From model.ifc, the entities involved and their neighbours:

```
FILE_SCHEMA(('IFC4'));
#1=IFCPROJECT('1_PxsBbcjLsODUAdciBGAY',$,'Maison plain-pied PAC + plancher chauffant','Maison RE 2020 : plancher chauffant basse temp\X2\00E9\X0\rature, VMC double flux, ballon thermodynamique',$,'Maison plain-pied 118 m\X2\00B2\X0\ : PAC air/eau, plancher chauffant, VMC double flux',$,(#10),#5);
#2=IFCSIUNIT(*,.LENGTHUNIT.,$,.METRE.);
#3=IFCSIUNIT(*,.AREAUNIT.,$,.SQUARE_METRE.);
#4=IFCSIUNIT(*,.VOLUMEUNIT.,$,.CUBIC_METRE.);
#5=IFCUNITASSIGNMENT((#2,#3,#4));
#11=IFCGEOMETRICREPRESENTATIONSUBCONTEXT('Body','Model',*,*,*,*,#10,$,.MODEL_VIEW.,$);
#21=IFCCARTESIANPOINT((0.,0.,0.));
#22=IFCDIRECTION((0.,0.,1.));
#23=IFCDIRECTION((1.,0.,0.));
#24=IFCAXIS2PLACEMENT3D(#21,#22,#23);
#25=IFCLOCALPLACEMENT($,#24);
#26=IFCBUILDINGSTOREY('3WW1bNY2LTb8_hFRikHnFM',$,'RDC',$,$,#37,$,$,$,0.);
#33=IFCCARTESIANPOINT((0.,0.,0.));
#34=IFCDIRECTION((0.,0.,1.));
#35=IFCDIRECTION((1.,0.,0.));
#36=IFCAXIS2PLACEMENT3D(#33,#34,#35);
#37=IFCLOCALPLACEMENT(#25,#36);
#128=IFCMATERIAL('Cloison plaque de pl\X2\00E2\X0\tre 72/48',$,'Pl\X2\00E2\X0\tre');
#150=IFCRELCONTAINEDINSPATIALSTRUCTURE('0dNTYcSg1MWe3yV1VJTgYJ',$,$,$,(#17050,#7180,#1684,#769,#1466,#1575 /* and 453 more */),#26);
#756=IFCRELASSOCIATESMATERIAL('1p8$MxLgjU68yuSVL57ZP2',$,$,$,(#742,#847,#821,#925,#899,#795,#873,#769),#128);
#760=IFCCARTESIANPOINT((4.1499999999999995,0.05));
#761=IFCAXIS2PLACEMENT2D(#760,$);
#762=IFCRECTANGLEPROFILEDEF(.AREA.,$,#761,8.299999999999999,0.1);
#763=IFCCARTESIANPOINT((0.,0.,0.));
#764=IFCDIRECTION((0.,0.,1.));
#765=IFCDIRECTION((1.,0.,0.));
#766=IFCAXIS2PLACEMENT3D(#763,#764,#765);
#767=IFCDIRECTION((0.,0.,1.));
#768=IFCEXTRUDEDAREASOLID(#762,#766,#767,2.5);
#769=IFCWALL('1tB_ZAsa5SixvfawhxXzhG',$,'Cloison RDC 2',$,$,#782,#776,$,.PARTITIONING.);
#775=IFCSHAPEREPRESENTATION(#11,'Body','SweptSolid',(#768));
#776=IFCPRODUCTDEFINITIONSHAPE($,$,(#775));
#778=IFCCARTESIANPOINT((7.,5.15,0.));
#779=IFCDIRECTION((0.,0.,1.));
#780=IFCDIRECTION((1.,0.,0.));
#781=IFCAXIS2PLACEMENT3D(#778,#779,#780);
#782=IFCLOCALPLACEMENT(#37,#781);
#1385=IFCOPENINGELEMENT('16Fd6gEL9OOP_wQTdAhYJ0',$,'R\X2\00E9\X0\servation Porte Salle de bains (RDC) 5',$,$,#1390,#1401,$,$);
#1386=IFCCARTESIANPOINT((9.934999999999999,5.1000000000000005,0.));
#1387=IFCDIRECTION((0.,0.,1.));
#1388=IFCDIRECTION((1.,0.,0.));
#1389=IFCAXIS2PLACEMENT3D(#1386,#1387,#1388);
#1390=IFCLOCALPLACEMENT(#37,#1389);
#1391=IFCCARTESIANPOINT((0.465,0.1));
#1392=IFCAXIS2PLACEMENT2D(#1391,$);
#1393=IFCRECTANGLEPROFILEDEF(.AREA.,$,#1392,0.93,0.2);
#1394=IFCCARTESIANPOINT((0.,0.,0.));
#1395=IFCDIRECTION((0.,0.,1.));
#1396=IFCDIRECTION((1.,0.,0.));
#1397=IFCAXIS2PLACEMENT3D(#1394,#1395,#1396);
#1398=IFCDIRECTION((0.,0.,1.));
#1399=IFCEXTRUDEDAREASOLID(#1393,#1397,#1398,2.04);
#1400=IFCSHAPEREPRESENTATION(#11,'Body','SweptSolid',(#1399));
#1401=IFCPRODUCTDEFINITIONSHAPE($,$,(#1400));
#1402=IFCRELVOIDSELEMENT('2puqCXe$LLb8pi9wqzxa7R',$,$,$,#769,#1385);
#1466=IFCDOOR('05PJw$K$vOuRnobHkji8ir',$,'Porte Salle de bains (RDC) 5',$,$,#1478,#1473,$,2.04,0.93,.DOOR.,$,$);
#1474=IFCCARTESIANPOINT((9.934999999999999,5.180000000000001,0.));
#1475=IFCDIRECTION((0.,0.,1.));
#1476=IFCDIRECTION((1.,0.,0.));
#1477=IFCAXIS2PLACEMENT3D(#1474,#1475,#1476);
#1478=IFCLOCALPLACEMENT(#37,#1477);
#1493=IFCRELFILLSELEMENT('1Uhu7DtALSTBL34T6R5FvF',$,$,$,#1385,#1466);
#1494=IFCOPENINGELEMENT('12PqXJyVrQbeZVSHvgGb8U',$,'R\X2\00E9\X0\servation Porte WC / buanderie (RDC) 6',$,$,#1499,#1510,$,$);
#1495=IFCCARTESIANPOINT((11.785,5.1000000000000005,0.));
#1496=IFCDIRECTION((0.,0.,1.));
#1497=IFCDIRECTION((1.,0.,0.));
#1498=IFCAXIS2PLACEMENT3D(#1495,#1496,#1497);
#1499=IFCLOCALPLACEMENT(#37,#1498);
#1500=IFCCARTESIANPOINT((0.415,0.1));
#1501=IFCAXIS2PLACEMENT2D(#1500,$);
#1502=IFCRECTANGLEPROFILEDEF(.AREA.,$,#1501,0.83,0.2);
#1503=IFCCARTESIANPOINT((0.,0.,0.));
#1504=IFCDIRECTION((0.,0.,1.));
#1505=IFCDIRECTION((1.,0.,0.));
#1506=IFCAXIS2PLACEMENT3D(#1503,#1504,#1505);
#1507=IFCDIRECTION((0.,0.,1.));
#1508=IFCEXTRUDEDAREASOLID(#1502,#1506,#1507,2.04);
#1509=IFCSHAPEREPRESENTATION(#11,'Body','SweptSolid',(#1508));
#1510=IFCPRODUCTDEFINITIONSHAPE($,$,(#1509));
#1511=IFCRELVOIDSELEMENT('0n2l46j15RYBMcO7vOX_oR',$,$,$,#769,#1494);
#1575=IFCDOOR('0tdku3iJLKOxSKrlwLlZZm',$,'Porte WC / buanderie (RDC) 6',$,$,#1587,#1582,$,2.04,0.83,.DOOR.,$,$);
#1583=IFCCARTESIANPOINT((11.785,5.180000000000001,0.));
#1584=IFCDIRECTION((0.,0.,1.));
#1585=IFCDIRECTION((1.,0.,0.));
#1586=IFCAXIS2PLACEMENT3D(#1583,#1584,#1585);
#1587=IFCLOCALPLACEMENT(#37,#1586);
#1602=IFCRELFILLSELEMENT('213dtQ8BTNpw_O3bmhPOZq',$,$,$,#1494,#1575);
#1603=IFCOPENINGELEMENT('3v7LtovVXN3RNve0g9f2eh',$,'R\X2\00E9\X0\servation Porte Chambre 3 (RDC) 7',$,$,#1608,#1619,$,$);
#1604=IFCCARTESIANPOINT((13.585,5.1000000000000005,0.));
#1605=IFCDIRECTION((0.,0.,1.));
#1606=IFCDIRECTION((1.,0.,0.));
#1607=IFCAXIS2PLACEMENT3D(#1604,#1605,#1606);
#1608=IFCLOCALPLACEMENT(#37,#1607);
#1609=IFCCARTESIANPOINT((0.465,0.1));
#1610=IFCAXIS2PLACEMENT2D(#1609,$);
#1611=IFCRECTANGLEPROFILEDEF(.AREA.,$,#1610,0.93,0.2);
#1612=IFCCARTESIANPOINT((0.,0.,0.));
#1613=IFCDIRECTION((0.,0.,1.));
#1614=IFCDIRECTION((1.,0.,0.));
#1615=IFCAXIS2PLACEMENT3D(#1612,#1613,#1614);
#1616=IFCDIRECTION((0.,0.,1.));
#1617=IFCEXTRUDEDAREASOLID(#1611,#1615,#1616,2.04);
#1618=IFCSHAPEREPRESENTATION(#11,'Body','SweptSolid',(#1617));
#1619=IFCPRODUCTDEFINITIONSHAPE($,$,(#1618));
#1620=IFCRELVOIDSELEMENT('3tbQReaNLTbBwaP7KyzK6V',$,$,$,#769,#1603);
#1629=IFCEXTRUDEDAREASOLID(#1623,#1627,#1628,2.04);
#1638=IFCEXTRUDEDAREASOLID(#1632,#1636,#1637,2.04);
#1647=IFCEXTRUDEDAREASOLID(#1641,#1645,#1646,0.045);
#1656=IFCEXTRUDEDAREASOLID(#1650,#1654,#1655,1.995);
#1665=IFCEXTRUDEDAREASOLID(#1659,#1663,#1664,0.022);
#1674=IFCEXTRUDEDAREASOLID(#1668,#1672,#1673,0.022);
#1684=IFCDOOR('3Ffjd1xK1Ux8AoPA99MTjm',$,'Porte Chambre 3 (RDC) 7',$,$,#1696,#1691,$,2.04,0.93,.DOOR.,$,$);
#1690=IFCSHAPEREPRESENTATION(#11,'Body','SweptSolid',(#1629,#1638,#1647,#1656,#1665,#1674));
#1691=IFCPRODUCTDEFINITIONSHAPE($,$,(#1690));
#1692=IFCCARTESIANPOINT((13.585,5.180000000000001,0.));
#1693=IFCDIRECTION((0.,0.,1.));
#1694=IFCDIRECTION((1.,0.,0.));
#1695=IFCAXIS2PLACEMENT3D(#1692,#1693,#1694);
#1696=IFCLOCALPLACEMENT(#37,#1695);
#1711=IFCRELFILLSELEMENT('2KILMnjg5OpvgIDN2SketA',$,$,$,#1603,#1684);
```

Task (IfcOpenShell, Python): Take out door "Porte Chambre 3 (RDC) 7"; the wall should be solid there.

```python
import ifcopenshell
import ifcopenshell.api.feature
import ifcopenshell.api.root
import ifcopenshell.geom
import ifcopenshell.util.shape

model = ifcopenshell.open("model.ifc")
settings = ifcopenshell.geom.settings()


def volume(element):
    """Net volume in cubic metres, openings subtracted."""
    shape = ifcopenshell.geom.create_shape(settings, element)
    return ifcopenshell.util.shape.get_volume(shape.geometry)


door = model.by_guid("3Ffjd1xK1Ux8AoPA99MTjm")
opening = door.FillsVoids[0].RelatingOpeningElement
wall = opening.VoidsElements[0].RelatingBuildingElement
before = volume(wall)

ifcopenshell.api.root.remove_product(model, product=door)
ifcopenshell.api.feature.remove_feature(model, feature=opening)

after = volume(wall)

print(f"wall volume {before:.3f} -> {after:.3f} m3")

model.write("model_rev.ifc")
```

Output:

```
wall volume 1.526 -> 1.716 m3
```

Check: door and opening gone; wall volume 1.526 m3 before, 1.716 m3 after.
